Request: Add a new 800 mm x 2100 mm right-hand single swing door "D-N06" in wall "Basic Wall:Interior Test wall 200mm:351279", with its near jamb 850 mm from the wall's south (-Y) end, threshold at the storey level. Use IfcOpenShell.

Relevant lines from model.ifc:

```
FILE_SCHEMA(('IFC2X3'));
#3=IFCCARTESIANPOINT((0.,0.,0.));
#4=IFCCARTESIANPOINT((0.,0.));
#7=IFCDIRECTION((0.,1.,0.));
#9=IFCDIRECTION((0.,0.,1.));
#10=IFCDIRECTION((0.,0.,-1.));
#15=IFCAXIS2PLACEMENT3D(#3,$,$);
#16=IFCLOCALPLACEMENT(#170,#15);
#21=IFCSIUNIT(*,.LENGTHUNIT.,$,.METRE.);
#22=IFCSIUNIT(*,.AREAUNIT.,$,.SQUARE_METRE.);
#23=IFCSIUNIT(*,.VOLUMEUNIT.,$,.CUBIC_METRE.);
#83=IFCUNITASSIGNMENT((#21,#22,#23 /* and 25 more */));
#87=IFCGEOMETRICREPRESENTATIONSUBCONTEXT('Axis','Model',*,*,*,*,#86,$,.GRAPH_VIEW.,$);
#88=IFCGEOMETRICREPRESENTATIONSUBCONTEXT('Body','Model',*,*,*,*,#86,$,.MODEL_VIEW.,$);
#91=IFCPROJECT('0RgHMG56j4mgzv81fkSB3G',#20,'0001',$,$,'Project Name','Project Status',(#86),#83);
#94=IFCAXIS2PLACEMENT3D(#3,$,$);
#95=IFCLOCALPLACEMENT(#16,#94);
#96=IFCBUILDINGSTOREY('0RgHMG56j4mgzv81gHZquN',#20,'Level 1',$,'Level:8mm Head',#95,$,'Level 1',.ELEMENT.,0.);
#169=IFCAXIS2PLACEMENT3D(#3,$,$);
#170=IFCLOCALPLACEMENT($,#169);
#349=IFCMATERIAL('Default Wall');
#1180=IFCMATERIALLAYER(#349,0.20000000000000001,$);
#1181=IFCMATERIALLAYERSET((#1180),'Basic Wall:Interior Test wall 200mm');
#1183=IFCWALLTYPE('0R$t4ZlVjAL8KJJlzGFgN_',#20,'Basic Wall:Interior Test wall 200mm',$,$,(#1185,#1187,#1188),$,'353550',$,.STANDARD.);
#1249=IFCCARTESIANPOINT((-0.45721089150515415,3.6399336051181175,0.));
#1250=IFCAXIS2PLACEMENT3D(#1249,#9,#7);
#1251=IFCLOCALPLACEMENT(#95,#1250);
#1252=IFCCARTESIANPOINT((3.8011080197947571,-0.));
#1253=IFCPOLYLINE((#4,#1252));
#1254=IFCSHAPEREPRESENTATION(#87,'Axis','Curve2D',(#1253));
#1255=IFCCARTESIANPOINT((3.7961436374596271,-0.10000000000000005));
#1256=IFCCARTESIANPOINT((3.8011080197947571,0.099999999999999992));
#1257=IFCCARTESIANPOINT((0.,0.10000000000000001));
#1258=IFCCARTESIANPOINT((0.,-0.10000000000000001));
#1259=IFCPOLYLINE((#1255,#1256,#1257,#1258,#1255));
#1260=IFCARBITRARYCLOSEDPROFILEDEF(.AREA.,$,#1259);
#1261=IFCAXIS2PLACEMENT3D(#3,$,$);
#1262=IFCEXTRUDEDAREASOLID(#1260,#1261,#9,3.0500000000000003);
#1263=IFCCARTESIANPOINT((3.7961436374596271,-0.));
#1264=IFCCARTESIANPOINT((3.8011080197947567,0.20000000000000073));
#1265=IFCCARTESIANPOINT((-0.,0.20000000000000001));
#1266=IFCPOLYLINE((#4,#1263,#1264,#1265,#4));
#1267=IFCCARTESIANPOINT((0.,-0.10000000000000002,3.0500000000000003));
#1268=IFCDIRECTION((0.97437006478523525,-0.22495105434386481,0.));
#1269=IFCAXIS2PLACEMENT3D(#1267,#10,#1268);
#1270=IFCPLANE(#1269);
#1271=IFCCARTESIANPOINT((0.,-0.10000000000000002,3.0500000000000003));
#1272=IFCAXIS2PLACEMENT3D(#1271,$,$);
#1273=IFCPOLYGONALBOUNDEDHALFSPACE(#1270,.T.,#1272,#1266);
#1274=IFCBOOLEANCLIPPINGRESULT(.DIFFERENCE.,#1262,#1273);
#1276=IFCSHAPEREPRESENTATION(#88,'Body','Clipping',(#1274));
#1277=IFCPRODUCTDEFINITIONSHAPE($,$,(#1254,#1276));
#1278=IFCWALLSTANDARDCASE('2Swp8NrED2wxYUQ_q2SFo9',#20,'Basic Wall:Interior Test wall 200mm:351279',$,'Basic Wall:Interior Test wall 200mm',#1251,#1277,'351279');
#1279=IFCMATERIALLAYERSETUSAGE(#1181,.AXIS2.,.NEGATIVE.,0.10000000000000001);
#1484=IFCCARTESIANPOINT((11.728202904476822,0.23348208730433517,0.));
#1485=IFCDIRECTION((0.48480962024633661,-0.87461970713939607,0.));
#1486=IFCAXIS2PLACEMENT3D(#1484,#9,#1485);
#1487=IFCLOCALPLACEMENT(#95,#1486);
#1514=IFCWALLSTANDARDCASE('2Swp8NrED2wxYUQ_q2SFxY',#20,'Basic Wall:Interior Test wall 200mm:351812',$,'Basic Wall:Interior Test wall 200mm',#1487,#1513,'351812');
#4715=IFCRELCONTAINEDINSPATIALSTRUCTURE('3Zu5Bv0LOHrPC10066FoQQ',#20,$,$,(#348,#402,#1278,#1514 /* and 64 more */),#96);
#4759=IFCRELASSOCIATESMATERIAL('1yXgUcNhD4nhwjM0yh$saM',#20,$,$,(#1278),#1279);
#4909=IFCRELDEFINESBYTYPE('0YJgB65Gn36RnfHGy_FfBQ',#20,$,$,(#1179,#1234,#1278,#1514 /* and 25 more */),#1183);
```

```python
import numpy as np
import ifcopenshell
import ifcopenshell.api.feature
import ifcopenshell.api.geometry
import ifcopenshell.api.root
import ifcopenshell.api.spatial
import ifcopenshell.api.type
import ifcopenshell.geom
import ifcopenshell.util.element
import ifcopenshell.util.placement
import ifcopenshell.util.representation
import ifcopenshell.util.shape
import ifcopenshell.util.unit

model = ifcopenshell.open("model.ifc")
unit_scale = ifcopenshell.util.unit.calculate_unit_scale(model)
settings = ifcopenshell.geom.settings()


def volume(element):
    """Net volume in cubic metres, openings subtracted."""
    shape = ifcopenshell.geom.create_shape(settings, element)
    return ifcopenshell.util.shape.get_volume(shape.geometry)


wall = model.by_guid("2Swp8NrED2wxYUQ_q2SFo9")
storey = ifcopenshell.util.element.get_container(wall, ifc_class="IfcBuildingStorey")
context = ifcopenshell.util.representation.get_context(model, "Model", "Body", "MODEL_VIEW")
before = volume(wall)

width, height, from_end, sill = 0.8, 2.1, 0.85, 0.0  # metres

# The wall runs along its own X axis, and the end named is its -X end.
wall_shape = ifcopenshell.geom.create_shape(settings, wall)
x, y, z = ifcopenshell.util.shape.get_vertices(wall_shape.geometry).T
start = x.min() + from_end
face, thickness = float(y.min()), float(y.max() - y.min())
wall_matrix = ifcopenshell.util.placement.get_local_placement(wall.ObjectPlacement)
level = ifcopenshell.util.placement.get_local_placement(storey.ObjectPlacement)[2, 3]


def in_wall(x, y):
    """Placement at x, y metres in the wall's axes, at sill height."""
    matrix = wall_matrix.copy()
    matrix[:, 3] = wall_matrix @ np.array([x / unit_scale, y / unit_scale, 0.0, 1.0])
    matrix[2, 3] = level + sill / unit_scale
    return matrix


# Opening: a box that overshoots both wall faces by 50 mm.
opening = ifcopenshell.api.root.create_entity(model, ifc_class="IfcOpeningElement")
box = ifcopenshell.api.geometry.add_wall_representation(
    model, context=context, length=width, height=height, thickness=thickness + 0.1
)
ifcopenshell.api.geometry.assign_representation(model, product=opening, representation=box)
ifcopenshell.api.geometry.edit_object_placement(model, product=opening, matrix=in_wall(start, face - 0.05), is_si=False)
ifcopenshell.api.feature.add_feature(model, feature=opening, element=wall)

door = ifcopenshell.api.root.create_entity(model, ifc_class="IfcDoor", name="D-N06")
door.OverallWidth, door.OverallHeight = width / unit_scale, height / unit_scale
body = ifcopenshell.api.geometry.add_door_representation(
    model,
    context=context,
    overall_width=door.OverallWidth,
    overall_height=door.OverallHeight,
    operation_type="SINGLE_SWING_RIGHT",
    lining_properties={"LiningDepth": thickness / unit_scale, "ThresholdDepth": thickness / unit_scale},
)
ifcopenshell.api.geometry.assign_representation(model, product=door, representation=body)
ifcopenshell.api.spatial.assign_container(model, products=[door], relating_structure=storey)
fills = ifcopenshell.api.feature.add_filling(model, opening=opening, element=door)
fills.OwnerHistory = door.OwnerHistory  # required in IFC2X3

# IFC2X3 keeps the operation on the door style.
style = ifcopenshell.api.root.create_entity(model, ifc_class="IfcDoorStyle", name="D-N06")
style.OperationType, style.ConstructionType = "SINGLE_SWING_RIGHT", "NOTDEFINED"
style.ParameterTakesPrecedence = style.Sizeable = False
ifcopenshell.api.type.assign_type(model, related_objects=[door], relating_type=style)

# The lining spans the wall, so the door starts at the wall face.
ifcopenshell.api.geometry.edit_object_placement(model, product=door, matrix=in_wall(start, face), is_si=False)

after = volume(wall)

print(f"wall volume {before:.3f} -> {after:.3f} m3")

model.write("model_v2.ifc")
```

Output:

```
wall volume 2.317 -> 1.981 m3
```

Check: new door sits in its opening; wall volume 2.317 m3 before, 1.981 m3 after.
